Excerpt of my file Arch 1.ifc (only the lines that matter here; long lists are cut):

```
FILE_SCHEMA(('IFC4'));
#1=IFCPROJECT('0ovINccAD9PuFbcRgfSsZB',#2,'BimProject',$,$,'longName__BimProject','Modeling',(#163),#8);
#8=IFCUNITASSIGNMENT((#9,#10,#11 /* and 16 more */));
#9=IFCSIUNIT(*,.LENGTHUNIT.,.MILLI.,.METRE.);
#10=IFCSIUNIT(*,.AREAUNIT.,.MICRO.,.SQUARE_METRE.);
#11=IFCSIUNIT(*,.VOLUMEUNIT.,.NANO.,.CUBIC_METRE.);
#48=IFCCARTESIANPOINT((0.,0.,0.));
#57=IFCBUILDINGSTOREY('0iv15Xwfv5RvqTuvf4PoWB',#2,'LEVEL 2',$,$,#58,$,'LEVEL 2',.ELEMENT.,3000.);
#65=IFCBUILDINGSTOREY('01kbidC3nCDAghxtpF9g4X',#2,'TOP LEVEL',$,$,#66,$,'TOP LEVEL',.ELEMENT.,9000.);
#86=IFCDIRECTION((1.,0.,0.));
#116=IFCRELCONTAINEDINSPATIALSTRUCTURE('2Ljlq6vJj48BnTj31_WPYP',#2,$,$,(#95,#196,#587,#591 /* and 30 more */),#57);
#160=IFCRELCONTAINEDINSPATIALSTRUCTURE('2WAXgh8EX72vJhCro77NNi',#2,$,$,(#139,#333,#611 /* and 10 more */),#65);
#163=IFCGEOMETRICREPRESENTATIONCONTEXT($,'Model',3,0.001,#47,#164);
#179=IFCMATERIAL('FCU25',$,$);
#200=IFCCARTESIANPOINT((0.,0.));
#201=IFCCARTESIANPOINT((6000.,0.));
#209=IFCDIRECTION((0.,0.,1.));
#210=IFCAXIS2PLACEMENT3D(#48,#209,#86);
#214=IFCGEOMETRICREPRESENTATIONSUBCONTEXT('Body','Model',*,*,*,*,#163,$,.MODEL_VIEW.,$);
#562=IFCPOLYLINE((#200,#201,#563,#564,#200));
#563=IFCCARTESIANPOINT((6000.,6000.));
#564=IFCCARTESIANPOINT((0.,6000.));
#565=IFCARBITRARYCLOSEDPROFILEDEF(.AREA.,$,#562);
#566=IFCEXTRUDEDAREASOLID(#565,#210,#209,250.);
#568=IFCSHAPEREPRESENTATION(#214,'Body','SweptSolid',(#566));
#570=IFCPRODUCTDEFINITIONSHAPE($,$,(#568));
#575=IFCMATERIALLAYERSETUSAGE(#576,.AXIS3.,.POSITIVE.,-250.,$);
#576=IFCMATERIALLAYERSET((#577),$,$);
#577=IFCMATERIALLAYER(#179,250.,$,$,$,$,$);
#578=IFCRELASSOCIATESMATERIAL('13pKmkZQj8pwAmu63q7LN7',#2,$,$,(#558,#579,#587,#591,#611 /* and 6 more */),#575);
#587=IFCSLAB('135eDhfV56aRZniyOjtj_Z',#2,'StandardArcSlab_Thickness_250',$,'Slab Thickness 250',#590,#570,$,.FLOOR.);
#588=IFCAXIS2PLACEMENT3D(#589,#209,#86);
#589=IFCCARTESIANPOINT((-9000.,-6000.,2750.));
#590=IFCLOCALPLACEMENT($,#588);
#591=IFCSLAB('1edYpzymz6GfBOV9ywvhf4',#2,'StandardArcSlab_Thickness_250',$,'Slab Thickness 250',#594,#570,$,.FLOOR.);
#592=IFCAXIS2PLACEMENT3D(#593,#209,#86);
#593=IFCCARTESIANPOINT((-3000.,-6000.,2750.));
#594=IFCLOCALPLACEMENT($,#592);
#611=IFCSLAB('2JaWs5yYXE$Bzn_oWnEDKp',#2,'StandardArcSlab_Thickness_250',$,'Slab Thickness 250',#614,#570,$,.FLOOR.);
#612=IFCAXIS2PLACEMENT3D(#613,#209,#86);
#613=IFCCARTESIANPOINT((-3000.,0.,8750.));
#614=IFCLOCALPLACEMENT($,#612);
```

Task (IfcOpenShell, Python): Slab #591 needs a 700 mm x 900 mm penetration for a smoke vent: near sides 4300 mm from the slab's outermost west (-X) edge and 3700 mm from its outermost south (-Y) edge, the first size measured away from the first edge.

```python
import numpy as np
import ifcopenshell
import ifcopenshell.api.feature
import ifcopenshell.api.geometry
import ifcopenshell.api.root
import ifcopenshell.geom
import ifcopenshell.util.placement
import ifcopenshell.util.representation
import ifcopenshell.util.shape
import ifcopenshell.util.unit

model = ifcopenshell.open("my file Arch 1.ifc")
unit_scale = ifcopenshell.util.unit.calculate_unit_scale(model)
settings = ifcopenshell.geom.settings()


def volume(element):
    """Net volume in cubic metres, openings subtracted."""
    shape = ifcopenshell.geom.create_shape(settings, element)
    return ifcopenshell.util.shape.get_volume(shape.geometry)


slab = model.by_guid("1edYpzymz6GfBOV9ywvhf4")
before = volume(slab)

# Extent in the slab's own axes, in metres. The edges named are its -X and -Y sides.
slab_shape = ifcopenshell.geom.create_shape(settings, slab)
vertices = ifcopenshell.util.shape.get_vertices(slab_shape.geometry)
x_min, y_min, bottom = vertices.min(axis=0)
top = vertices[:, 2].max()

opening = ifcopenshell.api.root.create_entity(model, ifc_class="IfcOpeningElement", name="Smoke vent opening", predefined_type="OPENING")
context = ifcopenshell.util.representation.get_context(model, "Model", "Body", "MODEL_VIEW")
width, depth = 0.7, 0.9
outline = [(0.0, 0.0), (width, 0.0), (width, depth), (0.0, depth), (0.0, 0.0)]
# Overshoot both faces by 50 mm so the cut is clean.
shape = ifcopenshell.api.geometry.add_slab_representation(
    model, context=context, depth=top - bottom + 0.1, polyline=outline
)
ifcopenshell.api.geometry.assign_representation(model, product=opening, representation=shape)

matrix = ifcopenshell.util.placement.get_local_placement(slab.ObjectPlacement)
matrix[:, 3] = matrix @ np.append(np.array([x_min + 4.3, y_min + 3.7, bottom - 0.05]) / unit_scale, 1.0)
ifcopenshell.api.geometry.edit_object_placement(model, product=opening, matrix=matrix, is_si=False)
ifcopenshell.api.feature.add_feature(model, feature=opening, element=slab)

after = volume(slab)

print(f"slab volume {before:.3f} -> {after:.3f} m3")

model.write("my file Arch 1_edited.ifc")
```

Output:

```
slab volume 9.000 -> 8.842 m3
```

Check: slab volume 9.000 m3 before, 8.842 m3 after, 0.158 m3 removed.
